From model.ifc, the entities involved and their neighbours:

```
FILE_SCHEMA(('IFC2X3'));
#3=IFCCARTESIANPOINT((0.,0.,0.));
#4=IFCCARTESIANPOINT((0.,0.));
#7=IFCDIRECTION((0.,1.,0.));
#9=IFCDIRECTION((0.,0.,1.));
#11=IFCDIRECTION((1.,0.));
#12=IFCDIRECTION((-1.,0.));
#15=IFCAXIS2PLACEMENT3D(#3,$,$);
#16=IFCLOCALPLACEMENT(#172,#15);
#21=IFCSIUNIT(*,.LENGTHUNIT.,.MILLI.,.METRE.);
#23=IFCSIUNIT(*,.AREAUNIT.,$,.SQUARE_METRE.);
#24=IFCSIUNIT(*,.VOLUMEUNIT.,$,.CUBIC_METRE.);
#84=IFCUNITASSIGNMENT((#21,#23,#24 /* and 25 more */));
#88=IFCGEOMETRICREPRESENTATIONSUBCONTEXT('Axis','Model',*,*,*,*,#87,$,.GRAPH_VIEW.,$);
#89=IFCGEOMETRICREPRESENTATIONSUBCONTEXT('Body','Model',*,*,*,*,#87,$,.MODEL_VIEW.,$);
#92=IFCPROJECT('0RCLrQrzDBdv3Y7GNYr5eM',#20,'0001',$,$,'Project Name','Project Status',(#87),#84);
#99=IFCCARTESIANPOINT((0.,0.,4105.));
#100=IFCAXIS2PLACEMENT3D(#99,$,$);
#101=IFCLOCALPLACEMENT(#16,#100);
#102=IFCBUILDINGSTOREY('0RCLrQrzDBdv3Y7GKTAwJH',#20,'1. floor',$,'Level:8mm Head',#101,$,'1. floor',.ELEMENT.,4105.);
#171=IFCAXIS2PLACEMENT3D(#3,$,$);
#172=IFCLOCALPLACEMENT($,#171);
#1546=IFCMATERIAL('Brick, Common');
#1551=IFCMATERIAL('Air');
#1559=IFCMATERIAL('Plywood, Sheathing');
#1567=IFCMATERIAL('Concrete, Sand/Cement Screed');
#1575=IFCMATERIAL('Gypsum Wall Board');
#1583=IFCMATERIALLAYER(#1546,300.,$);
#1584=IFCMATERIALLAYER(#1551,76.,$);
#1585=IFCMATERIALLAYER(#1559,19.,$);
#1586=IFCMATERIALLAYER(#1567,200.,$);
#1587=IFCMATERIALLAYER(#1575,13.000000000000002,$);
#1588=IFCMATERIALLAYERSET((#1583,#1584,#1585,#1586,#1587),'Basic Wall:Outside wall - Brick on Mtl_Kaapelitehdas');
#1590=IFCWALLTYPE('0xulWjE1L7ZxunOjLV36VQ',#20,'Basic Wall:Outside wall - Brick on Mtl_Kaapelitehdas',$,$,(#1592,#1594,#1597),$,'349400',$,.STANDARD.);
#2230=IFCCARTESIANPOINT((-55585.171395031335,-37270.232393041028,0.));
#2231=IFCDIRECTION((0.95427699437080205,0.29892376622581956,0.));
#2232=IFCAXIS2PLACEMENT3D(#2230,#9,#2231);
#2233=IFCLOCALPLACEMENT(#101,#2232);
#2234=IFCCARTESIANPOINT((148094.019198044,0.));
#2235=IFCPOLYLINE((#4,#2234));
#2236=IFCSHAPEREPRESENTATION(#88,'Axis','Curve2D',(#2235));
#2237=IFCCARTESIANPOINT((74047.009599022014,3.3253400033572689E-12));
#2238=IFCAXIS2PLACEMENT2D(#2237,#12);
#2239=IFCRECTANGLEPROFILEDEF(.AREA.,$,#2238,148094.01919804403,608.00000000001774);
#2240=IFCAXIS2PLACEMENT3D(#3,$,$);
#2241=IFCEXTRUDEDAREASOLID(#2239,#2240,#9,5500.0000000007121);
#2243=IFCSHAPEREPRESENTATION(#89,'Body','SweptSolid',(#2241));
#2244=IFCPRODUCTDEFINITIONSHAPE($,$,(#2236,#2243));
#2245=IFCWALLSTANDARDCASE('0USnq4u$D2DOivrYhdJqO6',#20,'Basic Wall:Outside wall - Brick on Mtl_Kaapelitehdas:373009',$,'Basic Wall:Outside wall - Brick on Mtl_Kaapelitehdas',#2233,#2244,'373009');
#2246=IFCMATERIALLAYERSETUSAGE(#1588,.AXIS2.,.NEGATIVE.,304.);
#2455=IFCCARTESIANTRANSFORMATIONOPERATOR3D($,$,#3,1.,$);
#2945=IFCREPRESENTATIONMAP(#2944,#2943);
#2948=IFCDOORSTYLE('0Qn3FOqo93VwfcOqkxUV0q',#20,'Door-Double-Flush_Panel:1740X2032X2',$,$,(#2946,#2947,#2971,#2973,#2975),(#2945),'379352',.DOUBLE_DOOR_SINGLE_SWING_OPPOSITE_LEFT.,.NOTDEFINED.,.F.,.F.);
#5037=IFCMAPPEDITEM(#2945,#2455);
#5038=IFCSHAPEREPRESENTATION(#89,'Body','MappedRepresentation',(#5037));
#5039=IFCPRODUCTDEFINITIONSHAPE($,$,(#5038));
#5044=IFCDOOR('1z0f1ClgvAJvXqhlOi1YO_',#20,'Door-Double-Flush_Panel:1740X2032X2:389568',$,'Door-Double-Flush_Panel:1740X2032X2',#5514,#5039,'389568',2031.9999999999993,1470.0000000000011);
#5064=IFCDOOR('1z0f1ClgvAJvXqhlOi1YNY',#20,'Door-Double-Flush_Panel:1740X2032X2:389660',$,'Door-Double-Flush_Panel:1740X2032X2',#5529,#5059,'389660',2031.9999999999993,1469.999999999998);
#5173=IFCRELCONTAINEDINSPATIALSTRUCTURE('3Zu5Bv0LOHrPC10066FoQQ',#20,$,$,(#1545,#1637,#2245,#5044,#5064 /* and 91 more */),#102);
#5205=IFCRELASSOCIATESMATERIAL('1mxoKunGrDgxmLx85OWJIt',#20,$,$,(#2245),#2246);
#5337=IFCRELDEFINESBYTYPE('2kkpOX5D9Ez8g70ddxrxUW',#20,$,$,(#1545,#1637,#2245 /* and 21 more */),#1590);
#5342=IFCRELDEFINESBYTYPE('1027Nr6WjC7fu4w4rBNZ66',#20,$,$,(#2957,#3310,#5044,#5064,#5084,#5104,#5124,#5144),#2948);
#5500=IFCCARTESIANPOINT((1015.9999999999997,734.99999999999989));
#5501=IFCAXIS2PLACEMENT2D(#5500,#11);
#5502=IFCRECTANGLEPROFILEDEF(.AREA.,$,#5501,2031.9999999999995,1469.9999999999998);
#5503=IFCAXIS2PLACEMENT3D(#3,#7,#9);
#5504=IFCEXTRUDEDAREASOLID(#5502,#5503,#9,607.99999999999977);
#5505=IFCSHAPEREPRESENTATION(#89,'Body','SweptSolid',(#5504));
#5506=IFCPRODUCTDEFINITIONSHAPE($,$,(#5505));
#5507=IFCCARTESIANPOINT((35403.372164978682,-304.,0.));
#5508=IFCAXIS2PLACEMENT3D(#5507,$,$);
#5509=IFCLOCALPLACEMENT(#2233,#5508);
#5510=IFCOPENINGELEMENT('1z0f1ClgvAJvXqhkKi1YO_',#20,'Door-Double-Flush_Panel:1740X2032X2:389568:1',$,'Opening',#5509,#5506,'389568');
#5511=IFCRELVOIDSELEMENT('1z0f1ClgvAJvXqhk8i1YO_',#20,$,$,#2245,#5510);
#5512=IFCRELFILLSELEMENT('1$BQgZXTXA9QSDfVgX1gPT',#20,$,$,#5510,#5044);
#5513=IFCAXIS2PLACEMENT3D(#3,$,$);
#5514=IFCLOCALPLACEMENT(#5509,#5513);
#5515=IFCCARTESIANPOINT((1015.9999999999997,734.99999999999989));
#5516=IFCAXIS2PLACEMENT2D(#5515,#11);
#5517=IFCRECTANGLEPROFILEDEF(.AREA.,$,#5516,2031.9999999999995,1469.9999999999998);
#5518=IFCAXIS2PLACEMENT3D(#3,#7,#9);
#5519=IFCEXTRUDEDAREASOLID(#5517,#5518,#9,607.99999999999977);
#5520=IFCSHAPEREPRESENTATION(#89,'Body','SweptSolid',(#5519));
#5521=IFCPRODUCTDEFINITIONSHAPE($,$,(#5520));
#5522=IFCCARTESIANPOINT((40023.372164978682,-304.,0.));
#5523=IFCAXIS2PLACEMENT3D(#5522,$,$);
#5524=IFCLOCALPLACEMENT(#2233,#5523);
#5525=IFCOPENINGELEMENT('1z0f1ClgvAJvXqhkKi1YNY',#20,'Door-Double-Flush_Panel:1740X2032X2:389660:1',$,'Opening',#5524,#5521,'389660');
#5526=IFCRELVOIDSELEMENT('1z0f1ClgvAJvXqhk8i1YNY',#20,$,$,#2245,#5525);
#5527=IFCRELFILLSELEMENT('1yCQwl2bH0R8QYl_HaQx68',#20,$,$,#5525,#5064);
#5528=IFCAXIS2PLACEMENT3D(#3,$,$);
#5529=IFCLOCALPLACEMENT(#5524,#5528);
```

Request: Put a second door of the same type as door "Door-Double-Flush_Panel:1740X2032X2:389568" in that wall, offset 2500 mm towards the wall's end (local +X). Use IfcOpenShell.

```python
import ifcopenshell
import ifcopenshell.api.feature
import ifcopenshell.api.geometry
import ifcopenshell.api.root
import ifcopenshell.geom
import ifcopenshell.util.element
import ifcopenshell.util.placement
import ifcopenshell.util.shape

model = ifcopenshell.open("model.ifc")
settings = ifcopenshell.geom.settings()


def volume(element):
    """Net volume in cubic metres, openings subtracted."""
    shape = ifcopenshell.geom.create_shape(settings, element)
    return ifcopenshell.util.shape.get_volume(shape.geometry)


def reuse_history(source, copy):
    """copy_class also copies each property set's owner history, people and application; keep the originals."""
    for rel in copy.IsDefinedBy:
        if rel.is_a("IfcRelDefinesByProperties") and (history := rel.RelatingPropertyDefinition.OwnerHistory):
            rel.RelatingPropertyDefinition.OwnerHistory = source.OwnerHistory
            ifcopenshell.util.element.remove_deep2(model, history)


door = model.by_guid("1z0f1ClgvAJvXqhlOi1YO_")
opening = door.FillsVoids[0].RelatingOpeningElement
wall = opening.VoidsElements[0].RelatingBuildingElement
before = volume(wall)
shift = ifcopenshell.util.placement.get_local_placement(wall.ObjectPlacement)[:3, 0] * 2500.0

# copy_class copies the void relationship, type, container and properties, but no geometry.
new_opening = ifcopenshell.api.root.copy_class(model, product=opening)
new_opening.Representation = ifcopenshell.util.element.copy_deep(
    model, opening.Representation, exclude=["IfcGeometricRepresentationContext", "IfcRepresentationMap"]
)
new_opening.Name = "Door-Double-Flush_Panel:1740X2032X2"
new_opening.Tag = None
new_door = ifcopenshell.api.root.copy_class(model, product=door)
new_door.Representation = ifcopenshell.util.element.copy_deep(
    model, door.Representation, exclude=["IfcGeometricRepresentationContext", "IfcRepresentationMap"]
)
new_door.Name = "Door-Double-Flush_Panel:1740X2032X2"
new_door.Tag = None
reuse_history(door, new_door)
fills = ifcopenshell.api.feature.add_filling(model, opening=new_opening, element=new_door)
fills.OwnerHistory = new_door.OwnerHistory  # required in IFC2X3

for old, new in ((opening, new_opening), (door, new_door)):
    matrix = ifcopenshell.util.placement.get_local_placement(old.ObjectPlacement)
    matrix[:3, 3] += shift
    ifcopenshell.api.geometry.edit_object_placement(model, product=new, matrix=matrix, is_si=False)

after = volume(wall)

print(f"wall volume {before:.3f} -> {after:.3f} m3")

model.write("model_updated.ifc")
```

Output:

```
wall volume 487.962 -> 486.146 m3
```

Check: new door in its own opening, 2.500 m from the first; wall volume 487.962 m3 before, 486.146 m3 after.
